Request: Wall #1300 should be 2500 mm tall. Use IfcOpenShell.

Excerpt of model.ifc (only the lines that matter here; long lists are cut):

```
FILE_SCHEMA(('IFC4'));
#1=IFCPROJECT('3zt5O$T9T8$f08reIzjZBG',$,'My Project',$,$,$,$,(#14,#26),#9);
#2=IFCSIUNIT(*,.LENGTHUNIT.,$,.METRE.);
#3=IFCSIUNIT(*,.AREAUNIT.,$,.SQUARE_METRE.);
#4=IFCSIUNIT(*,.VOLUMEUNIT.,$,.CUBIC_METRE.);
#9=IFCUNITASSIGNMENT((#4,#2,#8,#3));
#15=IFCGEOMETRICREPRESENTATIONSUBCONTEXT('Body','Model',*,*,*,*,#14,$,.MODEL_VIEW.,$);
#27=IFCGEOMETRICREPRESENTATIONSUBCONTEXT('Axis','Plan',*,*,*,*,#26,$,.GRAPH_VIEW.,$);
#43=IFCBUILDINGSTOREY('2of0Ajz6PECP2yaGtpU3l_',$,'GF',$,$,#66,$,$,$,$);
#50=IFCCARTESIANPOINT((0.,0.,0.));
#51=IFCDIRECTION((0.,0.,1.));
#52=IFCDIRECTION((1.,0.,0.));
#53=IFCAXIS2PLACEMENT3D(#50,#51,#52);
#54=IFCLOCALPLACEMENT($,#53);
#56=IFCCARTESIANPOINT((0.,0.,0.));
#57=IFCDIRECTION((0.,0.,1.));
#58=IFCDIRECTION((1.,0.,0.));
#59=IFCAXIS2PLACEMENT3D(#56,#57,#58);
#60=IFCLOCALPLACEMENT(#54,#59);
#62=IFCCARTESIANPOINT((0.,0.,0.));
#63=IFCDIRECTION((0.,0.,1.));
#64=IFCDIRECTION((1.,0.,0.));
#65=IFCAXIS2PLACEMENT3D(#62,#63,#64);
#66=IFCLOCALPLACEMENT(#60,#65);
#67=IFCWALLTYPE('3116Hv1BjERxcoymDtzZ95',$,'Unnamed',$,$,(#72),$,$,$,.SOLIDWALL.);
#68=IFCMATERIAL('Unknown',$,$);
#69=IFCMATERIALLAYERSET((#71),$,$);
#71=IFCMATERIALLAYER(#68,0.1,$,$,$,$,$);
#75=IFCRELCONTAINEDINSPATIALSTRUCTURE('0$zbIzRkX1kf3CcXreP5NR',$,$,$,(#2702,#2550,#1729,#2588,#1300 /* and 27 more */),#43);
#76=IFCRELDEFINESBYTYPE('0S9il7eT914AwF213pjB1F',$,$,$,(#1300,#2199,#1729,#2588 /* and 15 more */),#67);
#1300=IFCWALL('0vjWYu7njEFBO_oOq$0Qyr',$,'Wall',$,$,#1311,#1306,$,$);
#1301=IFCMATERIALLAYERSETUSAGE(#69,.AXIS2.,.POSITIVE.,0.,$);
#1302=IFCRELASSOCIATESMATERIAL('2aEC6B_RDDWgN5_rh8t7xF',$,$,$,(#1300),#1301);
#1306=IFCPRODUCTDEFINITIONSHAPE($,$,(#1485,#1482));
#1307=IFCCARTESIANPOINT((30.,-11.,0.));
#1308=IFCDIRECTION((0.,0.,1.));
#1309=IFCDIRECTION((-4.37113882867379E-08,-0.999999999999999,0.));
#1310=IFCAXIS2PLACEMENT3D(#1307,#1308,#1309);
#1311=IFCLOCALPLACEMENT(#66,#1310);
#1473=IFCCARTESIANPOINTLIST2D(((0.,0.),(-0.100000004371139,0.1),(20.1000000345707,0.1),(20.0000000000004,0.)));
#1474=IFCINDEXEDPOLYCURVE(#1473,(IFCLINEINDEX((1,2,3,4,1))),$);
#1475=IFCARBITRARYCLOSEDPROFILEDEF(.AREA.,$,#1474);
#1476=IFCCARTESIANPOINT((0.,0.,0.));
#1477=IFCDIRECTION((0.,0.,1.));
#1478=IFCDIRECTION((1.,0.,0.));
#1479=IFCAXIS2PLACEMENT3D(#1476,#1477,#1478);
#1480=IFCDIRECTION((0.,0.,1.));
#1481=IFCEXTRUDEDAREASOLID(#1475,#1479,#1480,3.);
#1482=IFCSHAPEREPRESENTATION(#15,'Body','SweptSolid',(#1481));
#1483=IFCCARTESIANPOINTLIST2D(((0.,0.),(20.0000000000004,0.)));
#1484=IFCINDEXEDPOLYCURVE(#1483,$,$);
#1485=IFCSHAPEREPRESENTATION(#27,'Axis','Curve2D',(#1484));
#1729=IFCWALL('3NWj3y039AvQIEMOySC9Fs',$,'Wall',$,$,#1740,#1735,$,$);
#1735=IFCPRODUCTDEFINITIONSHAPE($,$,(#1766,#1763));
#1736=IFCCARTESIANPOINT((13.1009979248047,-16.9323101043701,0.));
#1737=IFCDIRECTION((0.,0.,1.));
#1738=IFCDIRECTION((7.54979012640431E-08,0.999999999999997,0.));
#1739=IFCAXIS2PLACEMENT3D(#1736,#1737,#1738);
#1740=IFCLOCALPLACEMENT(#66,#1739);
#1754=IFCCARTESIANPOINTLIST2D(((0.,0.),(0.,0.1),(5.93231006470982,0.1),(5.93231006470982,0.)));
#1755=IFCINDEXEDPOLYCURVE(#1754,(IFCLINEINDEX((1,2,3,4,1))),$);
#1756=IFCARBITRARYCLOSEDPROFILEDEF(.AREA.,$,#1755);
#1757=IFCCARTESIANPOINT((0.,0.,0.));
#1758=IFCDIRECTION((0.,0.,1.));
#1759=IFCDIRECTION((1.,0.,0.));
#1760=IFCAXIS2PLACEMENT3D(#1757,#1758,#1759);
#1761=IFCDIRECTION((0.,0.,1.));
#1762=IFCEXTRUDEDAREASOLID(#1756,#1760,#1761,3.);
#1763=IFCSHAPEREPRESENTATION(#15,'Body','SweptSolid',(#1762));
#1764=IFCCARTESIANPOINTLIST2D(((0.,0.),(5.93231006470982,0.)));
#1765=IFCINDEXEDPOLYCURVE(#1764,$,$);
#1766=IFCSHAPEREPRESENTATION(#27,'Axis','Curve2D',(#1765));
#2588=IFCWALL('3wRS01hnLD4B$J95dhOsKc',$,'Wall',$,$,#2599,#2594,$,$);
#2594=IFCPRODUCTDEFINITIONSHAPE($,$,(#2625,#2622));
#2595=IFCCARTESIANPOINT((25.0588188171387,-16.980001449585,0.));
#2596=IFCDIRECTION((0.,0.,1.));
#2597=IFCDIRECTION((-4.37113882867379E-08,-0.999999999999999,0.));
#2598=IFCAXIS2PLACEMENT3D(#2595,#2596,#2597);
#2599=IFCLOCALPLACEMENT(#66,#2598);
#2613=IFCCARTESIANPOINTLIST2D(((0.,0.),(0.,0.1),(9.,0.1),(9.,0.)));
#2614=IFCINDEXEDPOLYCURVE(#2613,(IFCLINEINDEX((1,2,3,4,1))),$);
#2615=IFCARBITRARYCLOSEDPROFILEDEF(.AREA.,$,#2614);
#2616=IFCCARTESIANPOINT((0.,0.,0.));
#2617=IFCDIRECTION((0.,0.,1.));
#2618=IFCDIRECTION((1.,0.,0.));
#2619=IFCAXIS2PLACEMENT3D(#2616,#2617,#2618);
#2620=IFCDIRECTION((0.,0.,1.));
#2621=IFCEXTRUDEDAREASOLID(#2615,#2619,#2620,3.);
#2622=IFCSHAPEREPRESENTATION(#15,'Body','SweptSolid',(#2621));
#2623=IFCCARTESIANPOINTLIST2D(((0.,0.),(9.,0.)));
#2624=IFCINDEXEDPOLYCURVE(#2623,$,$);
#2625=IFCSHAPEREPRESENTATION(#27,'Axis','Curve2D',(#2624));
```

```python
import ifcopenshell
import ifcopenshell.geom
import ifcopenshell.util.representation
import ifcopenshell.util.shape
import ifcopenshell.util.unit

model = ifcopenshell.open("model.ifc")
unit_scale = ifcopenshell.util.unit.calculate_unit_scale(model)
settings = ifcopenshell.geom.settings()


def volume(element):
    """Net volume in cubic metres, openings subtracted."""
    shape = ifcopenshell.geom.create_shape(settings, element)
    return ifcopenshell.util.shape.get_volume(shape.geometry)


wall = model.by_guid("0vjWYu7njEFBO_oOq$0Qyr")
before = volume(wall)

body = ifcopenshell.util.representation.get_representation(wall, "Model", "Body")
solid = body.Items[0]
old_height = solid.Depth
solid.Depth = 2.5 / unit_scale
after = volume(wall)

print(f"height {old_height:g} -> {solid.Depth:g}, volume {before:.3f} -> {after:.3f} m3")

model.write("model_edited.ifc")
```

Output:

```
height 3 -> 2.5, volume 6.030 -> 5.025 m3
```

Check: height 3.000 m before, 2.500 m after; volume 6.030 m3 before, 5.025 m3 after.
